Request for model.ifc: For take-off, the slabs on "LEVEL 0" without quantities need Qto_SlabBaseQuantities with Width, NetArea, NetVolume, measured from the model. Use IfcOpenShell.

First a look at what the model holds.

```python
import ifcopenshell
import ifcopenshell.util.element
import ifcopenshell.util.unit

model = ifcopenshell.open("model.ifc")
print(model.schema)
for unit_type in ("LENGTHUNIT", "AREAUNIT", "VOLUMEUNIT"):
    print(unit_type, ifcopenshell.util.unit.calculate_unit_scale(model, unit_type))
storey = next(s for s in model.by_type("IfcBuildingStorey") if s.Name == "LEVEL 0")
slabs = [e for e in ifcopenshell.util.element.get_decomposition(storey) if e.is_a("IfcSlab")]
for e in sorted(slabs, key=lambda e: e.id()):
    print(e.id(), e.is_a(), e.Name, list(ifcopenshell.util.element.get_psets(e, qtos_only=True)), sep=" | ")
```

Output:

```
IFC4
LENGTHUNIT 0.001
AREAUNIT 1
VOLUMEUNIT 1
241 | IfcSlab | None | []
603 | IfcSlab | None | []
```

```python
import ifcopenshell
import ifcopenshell.api.pset
import ifcopenshell.geom
import ifcopenshell.util.element
import ifcopenshell.util.shape
import ifcopenshell.util.unit

model = ifcopenshell.open("model.ifc")
unit_scale = ifcopenshell.util.unit.calculate_unit_scale(model)
area_scale = ifcopenshell.util.unit.calculate_unit_scale(model, "AREAUNIT")
volume_scale = ifcopenshell.util.unit.calculate_unit_scale(model, "VOLUMEUNIT")
settings = ifcopenshell.geom.settings()

storey = next(s for s in model.by_type("IfcBuildingStorey") if s.Name == "LEVEL 0")
slabs = [e for e in ifcopenshell.util.element.get_decomposition(storey) if e.is_a("IfcSlab")]

for e in sorted(slabs, key=lambda e: e.id()):
    if ifcopenshell.util.element.get_psets(e, qtos_only=True, should_inherit=False):
        continue
    # Geometry comes back in metres, in the element's own axes.
    shape = ifcopenshell.geom.create_shape(settings, e)
    values = {
        "Width": ifcopenshell.util.shape.get_z(shape.geometry) / unit_scale,
        "NetArea": ifcopenshell.util.shape.get_footprint_area(shape.geometry) / area_scale,
        "NetVolume": ifcopenshell.util.shape.get_volume(shape.geometry) / volume_scale,
    }
    qto = ifcopenshell.api.pset.add_qto(model, product=e, name="Qto_SlabBaseQuantities")
    ifcopenshell.api.pset.edit_qto(model, qto=qto, properties=values)
    print(e.id(), {k: round(v, 3) for k, v in values.items()})

model.write("model_edited.ifc")
```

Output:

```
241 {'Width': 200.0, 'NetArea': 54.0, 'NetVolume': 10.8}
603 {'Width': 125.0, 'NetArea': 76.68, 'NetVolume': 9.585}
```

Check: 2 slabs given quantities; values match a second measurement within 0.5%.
